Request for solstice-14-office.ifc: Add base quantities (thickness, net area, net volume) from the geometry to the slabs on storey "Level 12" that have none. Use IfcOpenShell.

First a look at what the model holds.

```python
import ifcopenshell
import ifcopenshell.util.element
import ifcopenshell.util.unit

model = ifcopenshell.open("solstice-14-office.ifc")
print(model.schema)
for unit_type in ("LENGTHUNIT", "AREAUNIT", "VOLUMEUNIT"):
    print(unit_type, ifcopenshell.util.unit.calculate_unit_scale(model, unit_type))
storey = next(s for s in model.by_type("IfcBuildingStorey") if s.Name == "Level 12")
slabs = [e for e in ifcopenshell.util.element.get_decomposition(storey) if e.is_a("IfcSlab")]
for e in sorted(slabs, key=lambda e: e.id()):
    print(e.id(), e.is_a(), e.Name, list(ifcopenshell.util.element.get_psets(e, qtos_only=True)), sep=" | ")
```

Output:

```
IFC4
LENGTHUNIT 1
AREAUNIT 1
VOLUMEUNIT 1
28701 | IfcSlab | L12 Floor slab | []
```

```python
import ifcopenshell
import ifcopenshell.api.pset
import ifcopenshell.geom
import ifcopenshell.util.element
import ifcopenshell.util.shape
import ifcopenshell.util.unit

model = ifcopenshell.open("solstice-14-office.ifc")
unit_scale = ifcopenshell.util.unit.calculate_unit_scale(model)
area_scale = ifcopenshell.util.unit.calculate_unit_scale(model, "AREAUNIT")
volume_scale = ifcopenshell.util.unit.calculate_unit_scale(model, "VOLUMEUNIT")
settings = ifcopenshell.geom.settings()

storey = next(s for s in model.by_type("IfcBuildingStorey") if s.Name == "Level 12")
slabs = [e for e in ifcopenshell.util.element.get_decomposition(storey) if e.is_a("IfcSlab")]

for e in sorted(slabs, key=lambda e: e.id()):
    if ifcopenshell.util.element.get_psets(e, qtos_only=True, should_inherit=False):
        continue
    # Geometry comes back in metres, in the element's own axes.
    shape = ifcopenshell.geom.create_shape(settings, e)
    values = {
        "Width": ifcopenshell.util.shape.get_z(shape.geometry) / unit_scale,
        "NetArea": ifcopenshell.util.shape.get_footprint_area(shape.geometry) / area_scale,
        "NetVolume": ifcopenshell.util.shape.get_volume(shape.geometry) / volume_scale,
    }
    qto = ifcopenshell.api.pset.add_qto(model, product=e, name="Qto_SlabBaseQuantities")
    ifcopenshell.api.pset.edit_qto(model, qto=qto, properties=values)
    print(e.id(), {k: round(v, 3) for k, v in values.items()})

model.write("solstice-14-office_updated.ifc")
```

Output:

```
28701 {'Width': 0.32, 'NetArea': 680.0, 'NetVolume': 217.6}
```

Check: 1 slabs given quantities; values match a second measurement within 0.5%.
